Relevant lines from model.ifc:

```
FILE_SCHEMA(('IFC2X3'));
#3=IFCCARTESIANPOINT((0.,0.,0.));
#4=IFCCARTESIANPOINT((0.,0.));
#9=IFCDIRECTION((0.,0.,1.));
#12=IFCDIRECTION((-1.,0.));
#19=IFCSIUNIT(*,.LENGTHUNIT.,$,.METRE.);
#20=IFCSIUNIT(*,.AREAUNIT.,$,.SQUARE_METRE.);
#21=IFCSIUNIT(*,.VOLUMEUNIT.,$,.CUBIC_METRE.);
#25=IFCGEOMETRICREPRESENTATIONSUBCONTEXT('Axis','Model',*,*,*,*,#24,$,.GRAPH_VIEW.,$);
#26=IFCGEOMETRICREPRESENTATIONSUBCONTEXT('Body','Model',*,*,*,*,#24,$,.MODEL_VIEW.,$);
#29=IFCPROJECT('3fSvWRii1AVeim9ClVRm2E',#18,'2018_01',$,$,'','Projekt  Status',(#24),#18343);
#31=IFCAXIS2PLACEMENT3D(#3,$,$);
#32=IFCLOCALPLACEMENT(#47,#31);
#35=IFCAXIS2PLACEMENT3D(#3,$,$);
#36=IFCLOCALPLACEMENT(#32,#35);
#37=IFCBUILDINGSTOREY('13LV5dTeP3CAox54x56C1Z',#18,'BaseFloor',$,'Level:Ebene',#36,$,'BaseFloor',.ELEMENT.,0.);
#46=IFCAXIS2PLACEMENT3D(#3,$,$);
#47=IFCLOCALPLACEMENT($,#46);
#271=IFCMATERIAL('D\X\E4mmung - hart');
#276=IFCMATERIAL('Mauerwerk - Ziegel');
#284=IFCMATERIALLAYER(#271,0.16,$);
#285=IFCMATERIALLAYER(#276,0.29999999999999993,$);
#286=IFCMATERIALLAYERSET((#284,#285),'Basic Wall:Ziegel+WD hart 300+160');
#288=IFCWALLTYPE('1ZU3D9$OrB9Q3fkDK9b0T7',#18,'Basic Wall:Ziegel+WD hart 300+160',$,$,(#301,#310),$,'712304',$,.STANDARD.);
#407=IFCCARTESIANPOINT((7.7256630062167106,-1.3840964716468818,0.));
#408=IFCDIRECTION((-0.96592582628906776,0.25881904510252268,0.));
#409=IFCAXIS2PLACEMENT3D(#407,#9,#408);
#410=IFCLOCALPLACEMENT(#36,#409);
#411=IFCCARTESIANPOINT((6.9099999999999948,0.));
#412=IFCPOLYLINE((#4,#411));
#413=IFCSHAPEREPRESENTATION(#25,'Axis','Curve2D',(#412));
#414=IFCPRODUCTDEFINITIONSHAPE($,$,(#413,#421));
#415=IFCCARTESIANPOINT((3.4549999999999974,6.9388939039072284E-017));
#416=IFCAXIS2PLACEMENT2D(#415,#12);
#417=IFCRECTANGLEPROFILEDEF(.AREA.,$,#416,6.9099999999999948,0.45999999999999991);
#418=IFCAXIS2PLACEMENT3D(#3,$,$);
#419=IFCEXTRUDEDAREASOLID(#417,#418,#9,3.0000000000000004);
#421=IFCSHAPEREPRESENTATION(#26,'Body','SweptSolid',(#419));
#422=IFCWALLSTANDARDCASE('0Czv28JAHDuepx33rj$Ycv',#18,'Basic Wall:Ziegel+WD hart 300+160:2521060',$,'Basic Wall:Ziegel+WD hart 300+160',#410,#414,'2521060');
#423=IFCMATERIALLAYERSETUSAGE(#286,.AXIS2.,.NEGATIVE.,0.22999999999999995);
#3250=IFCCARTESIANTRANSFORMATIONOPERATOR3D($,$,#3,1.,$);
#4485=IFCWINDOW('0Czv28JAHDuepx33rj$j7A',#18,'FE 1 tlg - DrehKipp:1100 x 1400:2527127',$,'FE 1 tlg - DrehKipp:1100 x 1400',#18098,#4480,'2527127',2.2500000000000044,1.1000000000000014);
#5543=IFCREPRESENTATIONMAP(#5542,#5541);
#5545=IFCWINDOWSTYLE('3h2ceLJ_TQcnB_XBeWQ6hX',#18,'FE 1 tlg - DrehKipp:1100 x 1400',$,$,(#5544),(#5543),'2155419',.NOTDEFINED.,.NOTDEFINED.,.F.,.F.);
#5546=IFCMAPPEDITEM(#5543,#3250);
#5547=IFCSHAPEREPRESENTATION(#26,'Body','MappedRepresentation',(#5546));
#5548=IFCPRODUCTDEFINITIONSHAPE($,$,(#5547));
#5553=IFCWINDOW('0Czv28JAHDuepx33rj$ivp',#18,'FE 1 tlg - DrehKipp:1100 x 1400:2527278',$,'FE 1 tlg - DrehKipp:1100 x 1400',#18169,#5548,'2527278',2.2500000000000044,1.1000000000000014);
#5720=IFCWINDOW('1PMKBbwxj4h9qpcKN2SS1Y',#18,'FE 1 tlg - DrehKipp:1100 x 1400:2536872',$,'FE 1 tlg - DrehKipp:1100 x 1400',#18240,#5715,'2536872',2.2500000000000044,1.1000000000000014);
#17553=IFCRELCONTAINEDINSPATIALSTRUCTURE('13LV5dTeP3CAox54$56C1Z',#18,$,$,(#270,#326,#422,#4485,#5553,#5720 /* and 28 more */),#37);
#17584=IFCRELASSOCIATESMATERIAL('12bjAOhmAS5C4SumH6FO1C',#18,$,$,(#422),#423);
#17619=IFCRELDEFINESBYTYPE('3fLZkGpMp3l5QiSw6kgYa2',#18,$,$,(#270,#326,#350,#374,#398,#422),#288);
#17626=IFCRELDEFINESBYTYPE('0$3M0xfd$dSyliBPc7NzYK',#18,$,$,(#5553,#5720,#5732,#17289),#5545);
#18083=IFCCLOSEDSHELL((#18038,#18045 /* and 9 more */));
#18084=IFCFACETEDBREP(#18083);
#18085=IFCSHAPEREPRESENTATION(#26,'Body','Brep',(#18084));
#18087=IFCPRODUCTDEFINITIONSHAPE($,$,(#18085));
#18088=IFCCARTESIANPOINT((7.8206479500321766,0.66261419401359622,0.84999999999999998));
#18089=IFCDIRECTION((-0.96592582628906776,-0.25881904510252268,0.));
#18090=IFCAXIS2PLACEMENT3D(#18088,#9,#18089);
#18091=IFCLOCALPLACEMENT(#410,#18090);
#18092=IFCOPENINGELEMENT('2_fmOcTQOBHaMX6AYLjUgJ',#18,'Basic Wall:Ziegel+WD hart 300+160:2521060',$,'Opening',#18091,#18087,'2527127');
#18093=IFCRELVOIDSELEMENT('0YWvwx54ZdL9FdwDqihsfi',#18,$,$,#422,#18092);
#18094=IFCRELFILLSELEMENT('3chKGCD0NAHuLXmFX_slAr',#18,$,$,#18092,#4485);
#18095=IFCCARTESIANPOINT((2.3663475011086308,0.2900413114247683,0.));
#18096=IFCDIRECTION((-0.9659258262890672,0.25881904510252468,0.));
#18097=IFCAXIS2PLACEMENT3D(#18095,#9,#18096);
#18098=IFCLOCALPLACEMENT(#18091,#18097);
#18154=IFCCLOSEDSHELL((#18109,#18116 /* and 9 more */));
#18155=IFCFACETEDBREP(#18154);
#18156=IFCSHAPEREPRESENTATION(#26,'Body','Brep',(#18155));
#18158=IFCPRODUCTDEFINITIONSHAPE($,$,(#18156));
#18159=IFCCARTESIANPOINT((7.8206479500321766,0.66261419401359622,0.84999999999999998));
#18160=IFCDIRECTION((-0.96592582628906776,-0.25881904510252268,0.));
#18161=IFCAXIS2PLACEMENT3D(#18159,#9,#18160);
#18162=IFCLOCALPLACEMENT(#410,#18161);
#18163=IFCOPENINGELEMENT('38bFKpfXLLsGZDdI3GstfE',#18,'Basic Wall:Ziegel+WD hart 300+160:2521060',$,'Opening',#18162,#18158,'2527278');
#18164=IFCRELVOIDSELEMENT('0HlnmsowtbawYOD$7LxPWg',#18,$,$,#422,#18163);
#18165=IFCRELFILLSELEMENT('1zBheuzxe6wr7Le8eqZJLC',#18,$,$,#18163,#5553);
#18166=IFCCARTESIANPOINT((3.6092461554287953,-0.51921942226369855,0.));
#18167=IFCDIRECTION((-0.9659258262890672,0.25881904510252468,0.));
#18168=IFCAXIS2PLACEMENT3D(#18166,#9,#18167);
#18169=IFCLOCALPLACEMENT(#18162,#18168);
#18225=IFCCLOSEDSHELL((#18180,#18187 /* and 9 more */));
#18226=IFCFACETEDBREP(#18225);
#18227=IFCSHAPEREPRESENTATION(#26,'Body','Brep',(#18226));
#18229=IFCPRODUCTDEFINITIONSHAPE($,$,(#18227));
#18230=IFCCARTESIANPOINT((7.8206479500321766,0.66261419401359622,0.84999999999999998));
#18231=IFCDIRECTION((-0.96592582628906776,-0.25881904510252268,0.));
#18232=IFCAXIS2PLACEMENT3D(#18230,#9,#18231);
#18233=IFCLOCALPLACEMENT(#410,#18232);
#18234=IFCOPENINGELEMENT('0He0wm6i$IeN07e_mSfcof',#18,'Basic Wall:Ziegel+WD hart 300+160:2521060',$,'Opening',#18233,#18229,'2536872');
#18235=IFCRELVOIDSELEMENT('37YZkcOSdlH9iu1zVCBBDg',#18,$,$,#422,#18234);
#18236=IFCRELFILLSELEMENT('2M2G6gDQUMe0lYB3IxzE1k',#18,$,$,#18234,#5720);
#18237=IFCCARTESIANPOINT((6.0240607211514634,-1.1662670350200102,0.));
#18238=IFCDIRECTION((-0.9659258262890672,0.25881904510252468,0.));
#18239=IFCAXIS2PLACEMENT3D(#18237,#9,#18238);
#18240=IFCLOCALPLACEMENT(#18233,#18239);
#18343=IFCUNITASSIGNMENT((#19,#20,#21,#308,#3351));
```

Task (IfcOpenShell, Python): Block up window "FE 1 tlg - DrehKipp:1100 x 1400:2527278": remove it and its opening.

```python
import ifcopenshell
import ifcopenshell.api.feature
import ifcopenshell.api.root
import ifcopenshell.geom
import ifcopenshell.util.shape

model = ifcopenshell.open("model.ifc")
settings = ifcopenshell.geom.settings()


def volume(element):
    """Net volume in cubic metres, openings subtracted."""
    shape = ifcopenshell.geom.create_shape(settings, element)
    return ifcopenshell.util.shape.get_volume(shape.geometry)


window = model.by_id(5553)
opening = window.FillsVoids[0].RelatingOpeningElement
wall = opening.VoidsElements[0].RelatingBuildingElement
before = volume(wall)

ifcopenshell.api.root.remove_product(model, product=window)
ifcopenshell.api.feature.remove_feature(model, feature=opening)

after = volume(wall)

print(f"wall volume {before:.3f} -> {after:.3f} m3")

model.write("model-out.ifc")
```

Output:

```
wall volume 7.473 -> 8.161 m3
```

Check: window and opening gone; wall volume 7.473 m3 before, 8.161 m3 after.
